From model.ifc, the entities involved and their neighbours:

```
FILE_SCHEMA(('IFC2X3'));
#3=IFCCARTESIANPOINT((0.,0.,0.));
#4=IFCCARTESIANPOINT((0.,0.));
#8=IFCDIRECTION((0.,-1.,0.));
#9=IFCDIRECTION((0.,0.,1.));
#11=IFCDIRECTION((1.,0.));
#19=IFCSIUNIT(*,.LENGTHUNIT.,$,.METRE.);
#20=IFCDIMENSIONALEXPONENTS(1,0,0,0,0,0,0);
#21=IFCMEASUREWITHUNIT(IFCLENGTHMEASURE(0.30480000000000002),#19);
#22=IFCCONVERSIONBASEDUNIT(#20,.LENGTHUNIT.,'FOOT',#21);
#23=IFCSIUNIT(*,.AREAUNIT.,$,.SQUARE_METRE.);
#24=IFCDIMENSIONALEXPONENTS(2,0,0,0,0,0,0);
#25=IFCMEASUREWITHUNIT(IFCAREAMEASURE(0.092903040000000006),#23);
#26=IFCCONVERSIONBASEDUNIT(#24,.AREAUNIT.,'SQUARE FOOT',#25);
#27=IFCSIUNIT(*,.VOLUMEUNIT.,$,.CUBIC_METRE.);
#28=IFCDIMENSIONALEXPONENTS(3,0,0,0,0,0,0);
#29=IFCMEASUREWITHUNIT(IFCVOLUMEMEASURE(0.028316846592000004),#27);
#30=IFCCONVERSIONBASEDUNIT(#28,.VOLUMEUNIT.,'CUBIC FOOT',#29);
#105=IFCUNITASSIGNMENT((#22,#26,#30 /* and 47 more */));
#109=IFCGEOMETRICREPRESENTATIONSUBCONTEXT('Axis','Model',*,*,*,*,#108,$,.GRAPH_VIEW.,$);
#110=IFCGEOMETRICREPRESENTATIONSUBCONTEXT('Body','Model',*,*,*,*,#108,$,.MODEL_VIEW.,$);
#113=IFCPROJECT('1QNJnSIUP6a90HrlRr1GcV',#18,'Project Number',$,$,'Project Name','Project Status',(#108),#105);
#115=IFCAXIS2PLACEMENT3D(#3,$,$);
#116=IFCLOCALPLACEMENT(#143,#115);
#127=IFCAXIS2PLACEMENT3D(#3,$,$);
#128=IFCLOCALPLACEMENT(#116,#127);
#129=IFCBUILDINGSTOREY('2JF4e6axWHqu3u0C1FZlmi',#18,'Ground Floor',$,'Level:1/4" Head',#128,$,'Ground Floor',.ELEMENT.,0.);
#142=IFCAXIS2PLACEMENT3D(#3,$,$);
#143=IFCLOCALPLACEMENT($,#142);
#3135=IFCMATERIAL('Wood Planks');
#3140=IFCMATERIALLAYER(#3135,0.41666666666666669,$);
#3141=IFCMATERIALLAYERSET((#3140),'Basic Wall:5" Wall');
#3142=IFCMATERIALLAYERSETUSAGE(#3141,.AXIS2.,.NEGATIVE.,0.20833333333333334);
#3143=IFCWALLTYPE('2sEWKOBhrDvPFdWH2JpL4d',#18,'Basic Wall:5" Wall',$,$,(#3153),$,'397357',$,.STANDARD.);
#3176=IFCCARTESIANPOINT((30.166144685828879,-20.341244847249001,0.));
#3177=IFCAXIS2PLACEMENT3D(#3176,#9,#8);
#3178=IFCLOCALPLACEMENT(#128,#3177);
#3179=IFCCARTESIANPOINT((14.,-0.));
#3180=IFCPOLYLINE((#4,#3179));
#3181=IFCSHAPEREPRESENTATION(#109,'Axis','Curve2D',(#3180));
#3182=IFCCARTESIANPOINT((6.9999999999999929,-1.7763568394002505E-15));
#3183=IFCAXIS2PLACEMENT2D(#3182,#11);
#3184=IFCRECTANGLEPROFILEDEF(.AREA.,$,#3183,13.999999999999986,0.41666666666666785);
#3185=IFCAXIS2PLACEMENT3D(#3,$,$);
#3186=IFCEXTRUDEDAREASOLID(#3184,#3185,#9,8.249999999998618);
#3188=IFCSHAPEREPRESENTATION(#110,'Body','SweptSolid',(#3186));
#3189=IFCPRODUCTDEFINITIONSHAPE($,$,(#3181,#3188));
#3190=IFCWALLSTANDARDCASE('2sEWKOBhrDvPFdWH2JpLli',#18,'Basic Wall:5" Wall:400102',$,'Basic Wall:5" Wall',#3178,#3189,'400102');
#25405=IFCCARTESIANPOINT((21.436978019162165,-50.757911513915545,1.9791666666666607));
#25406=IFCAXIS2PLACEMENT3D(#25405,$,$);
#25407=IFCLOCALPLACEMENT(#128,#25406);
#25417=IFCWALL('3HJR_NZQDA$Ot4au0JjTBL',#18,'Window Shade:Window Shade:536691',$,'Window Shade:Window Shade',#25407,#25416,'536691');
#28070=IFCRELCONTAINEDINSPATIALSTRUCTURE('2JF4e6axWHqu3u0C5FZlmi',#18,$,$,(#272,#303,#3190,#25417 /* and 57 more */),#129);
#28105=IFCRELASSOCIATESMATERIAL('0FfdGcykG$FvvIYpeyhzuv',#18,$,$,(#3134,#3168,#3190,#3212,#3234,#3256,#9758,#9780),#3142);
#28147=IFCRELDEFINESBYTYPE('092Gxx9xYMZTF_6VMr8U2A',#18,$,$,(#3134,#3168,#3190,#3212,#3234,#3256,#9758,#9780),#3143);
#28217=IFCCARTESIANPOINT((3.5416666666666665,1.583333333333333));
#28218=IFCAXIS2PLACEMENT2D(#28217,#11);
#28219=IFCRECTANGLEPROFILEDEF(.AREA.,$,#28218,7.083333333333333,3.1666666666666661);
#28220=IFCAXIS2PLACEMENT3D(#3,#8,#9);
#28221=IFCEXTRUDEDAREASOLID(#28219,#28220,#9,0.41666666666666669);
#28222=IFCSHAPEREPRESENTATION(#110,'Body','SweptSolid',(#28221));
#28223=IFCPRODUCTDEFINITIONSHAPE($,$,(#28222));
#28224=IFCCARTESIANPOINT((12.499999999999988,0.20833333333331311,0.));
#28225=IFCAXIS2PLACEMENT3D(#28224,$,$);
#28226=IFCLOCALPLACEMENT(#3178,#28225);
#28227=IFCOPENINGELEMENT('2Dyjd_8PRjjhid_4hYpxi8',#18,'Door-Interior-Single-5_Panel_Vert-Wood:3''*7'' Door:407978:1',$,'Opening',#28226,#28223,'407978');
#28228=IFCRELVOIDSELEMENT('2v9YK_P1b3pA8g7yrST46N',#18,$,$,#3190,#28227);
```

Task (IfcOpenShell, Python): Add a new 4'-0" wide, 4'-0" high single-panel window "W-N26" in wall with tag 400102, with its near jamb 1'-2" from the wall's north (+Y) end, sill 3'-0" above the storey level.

```python
import numpy as np
import ifcopenshell
import ifcopenshell.api.feature
import ifcopenshell.api.geometry
import ifcopenshell.api.root
import ifcopenshell.api.spatial
import ifcopenshell.api.type
import ifcopenshell.geom
import ifcopenshell.util.element
import ifcopenshell.util.placement
import ifcopenshell.util.representation
import ifcopenshell.util.shape
import ifcopenshell.util.unit

model = ifcopenshell.open("model.ifc")
unit_scale = ifcopenshell.util.unit.calculate_unit_scale(model)
settings = ifcopenshell.geom.settings()


def volume(element):
    """Net volume in cubic metres, openings subtracted."""
    shape = ifcopenshell.geom.create_shape(settings, element)
    return ifcopenshell.util.shape.get_volume(shape.geometry)


wall = model.by_guid("2sEWKOBhrDvPFdWH2JpLli")
storey = ifcopenshell.util.element.get_container(wall, ifc_class="IfcBuildingStorey")
context = ifcopenshell.util.representation.get_context(model, "Model", "Body", "MODEL_VIEW")
before = volume(wall)

width, height, from_end, sill = 1.2192, 1.2192, 0.3556, 0.9144  # metres

# The wall runs along its own X axis, and the end named is its -X end.
wall_shape = ifcopenshell.geom.create_shape(settings, wall)
x, y, z = ifcopenshell.util.shape.get_vertices(wall_shape.geometry).T
start = x.min() + from_end
face, thickness = float(y.min()), float(y.max() - y.min())
wall_matrix = ifcopenshell.util.placement.get_local_placement(wall.ObjectPlacement)
level = ifcopenshell.util.placement.get_local_placement(storey.ObjectPlacement)[2, 3]


def in_wall(x, y):
    """Placement at x, y metres in the wall's axes, at sill height."""
    matrix = wall_matrix.copy()
    matrix[:, 3] = wall_matrix @ np.array([x / unit_scale, y / unit_scale, 0.0, 1.0])
    matrix[2, 3] = level + sill / unit_scale
    return matrix


# Opening: a box that overshoots both wall faces by 50 mm.
opening = ifcopenshell.api.root.create_entity(model, ifc_class="IfcOpeningElement")
box = ifcopenshell.api.geometry.add_wall_representation(
    model, context=context, length=width, height=height, thickness=thickness + 0.1
)
ifcopenshell.api.geometry.assign_representation(model, product=opening, representation=box)
ifcopenshell.api.geometry.edit_object_placement(model, product=opening, matrix=in_wall(start, face - 0.05), is_si=False)
ifcopenshell.api.feature.add_feature(model, feature=opening, element=wall)

window = ifcopenshell.api.root.create_entity(model, ifc_class="IfcWindow", name="W-N26")
window.OverallWidth, window.OverallHeight = width / unit_scale, height / unit_scale
body = ifcopenshell.api.geometry.add_window_representation(
    model,
    context=context,
    overall_width=window.OverallWidth,
    overall_height=window.OverallHeight,
    partition_type="SINGLE_PANEL",
)
ifcopenshell.api.geometry.assign_representation(model, product=window, representation=body)
ifcopenshell.api.spatial.assign_container(model, products=[window], relating_structure=storey)
fills = ifcopenshell.api.feature.add_filling(model, opening=opening, element=window)
fills.OwnerHistory = window.OwnerHistory  # required in IFC2X3

# IFC2X3 keeps the operation on the window style.
style = ifcopenshell.api.root.create_entity(model, ifc_class="IfcWindowStyle", name="W-N26")
style.OperationType, style.ConstructionType = "SINGLE_PANEL", "NOTDEFINED"
style.ParameterTakesPrecedence = style.Sizeable = False
ifcopenshell.api.type.assign_type(model, related_objects=[window], relating_type=style)

# Centre the window in the wall's thickness.
ifcopenshell.api.geometry.edit_object_placement(model, product=window, matrix=in_wall(start, face), is_si=False)
window_shape = ifcopenshell.geom.create_shape(settings, window)
depth = ifcopenshell.util.shape.get_vertices(window_shape.geometry)[:, 1]
offset = face + thickness / 2 - (depth.min() + depth.max()) / 2
ifcopenshell.api.geometry.edit_object_placement(model, product=window, matrix=in_wall(start, offset), is_si=False)

after = volume(wall)

print(f"wall volume {before:.3f} -> {after:.3f} m3")

model.write("model_updated.ifc")
```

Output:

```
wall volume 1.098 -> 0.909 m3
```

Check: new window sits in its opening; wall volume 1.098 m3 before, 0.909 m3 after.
